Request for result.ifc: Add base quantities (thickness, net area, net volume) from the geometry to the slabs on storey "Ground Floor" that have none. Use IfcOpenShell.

First a look at what the model holds.

```python
import ifcopenshell
import ifcopenshell.util.element
import ifcopenshell.util.unit

model = ifcopenshell.open("result.ifc")
print(model.schema)
for unit_type in ("LENGTHUNIT", "AREAUNIT", "VOLUMEUNIT"):
    print(unit_type, ifcopenshell.util.unit.calculate_unit_scale(model, unit_type))
storey = next(s for s in model.by_type("IfcBuildingStorey") if s.Name == "Ground Floor")
slabs = [e for e in ifcopenshell.util.element.get_decomposition(storey) if e.is_a("IfcSlab")]
for e in sorted(slabs, key=lambda e: e.id()):
    print(e.id(), e.is_a(), e.Name, list(ifcopenshell.util.element.get_psets(e, qtos_only=True)), sep=" | ")
```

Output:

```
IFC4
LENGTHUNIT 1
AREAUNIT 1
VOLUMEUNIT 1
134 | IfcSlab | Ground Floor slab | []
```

```python
import ifcopenshell
import ifcopenshell.api.pset
import ifcopenshell.geom
import ifcopenshell.util.element
import ifcopenshell.util.shape
import ifcopenshell.util.unit

model = ifcopenshell.open("result.ifc")
unit_scale = ifcopenshell.util.unit.calculate_unit_scale(model)
area_scale = ifcopenshell.util.unit.calculate_unit_scale(model, "AREAUNIT")
volume_scale = ifcopenshell.util.unit.calculate_unit_scale(model, "VOLUMEUNIT")
settings = ifcopenshell.geom.settings()

storey = next(s for s in model.by_type("IfcBuildingStorey") if s.Name == "Ground Floor")
slabs = [e for e in ifcopenshell.util.element.get_decomposition(storey) if e.is_a("IfcSlab")]

for e in sorted(slabs, key=lambda e: e.id()):
    if ifcopenshell.util.element.get_psets(e, qtos_only=True, should_inherit=False):
        continue
    # Geometry comes back in metres, in the element's own axes.
    shape = ifcopenshell.geom.create_shape(settings, e)
    values = {
        "Width": ifcopenshell.util.shape.get_z(shape.geometry) / unit_scale,
        "NetArea": ifcopenshell.util.shape.get_footprint_area(shape.geometry) / area_scale,
        "NetVolume": ifcopenshell.util.shape.get_volume(shape.geometry) / volume_scale,
    }
    qto = ifcopenshell.api.pset.add_qto(model, product=e, name="Qto_SlabBaseQuantities")
    ifcopenshell.api.pset.edit_qto(model, qto=qto, properties=values)
    print(e.id(), {k: round(v, 3) for k, v in values.items()})

model.write("result_rev.ifc")
```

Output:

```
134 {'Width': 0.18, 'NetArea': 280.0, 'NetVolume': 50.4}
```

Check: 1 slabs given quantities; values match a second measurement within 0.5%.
